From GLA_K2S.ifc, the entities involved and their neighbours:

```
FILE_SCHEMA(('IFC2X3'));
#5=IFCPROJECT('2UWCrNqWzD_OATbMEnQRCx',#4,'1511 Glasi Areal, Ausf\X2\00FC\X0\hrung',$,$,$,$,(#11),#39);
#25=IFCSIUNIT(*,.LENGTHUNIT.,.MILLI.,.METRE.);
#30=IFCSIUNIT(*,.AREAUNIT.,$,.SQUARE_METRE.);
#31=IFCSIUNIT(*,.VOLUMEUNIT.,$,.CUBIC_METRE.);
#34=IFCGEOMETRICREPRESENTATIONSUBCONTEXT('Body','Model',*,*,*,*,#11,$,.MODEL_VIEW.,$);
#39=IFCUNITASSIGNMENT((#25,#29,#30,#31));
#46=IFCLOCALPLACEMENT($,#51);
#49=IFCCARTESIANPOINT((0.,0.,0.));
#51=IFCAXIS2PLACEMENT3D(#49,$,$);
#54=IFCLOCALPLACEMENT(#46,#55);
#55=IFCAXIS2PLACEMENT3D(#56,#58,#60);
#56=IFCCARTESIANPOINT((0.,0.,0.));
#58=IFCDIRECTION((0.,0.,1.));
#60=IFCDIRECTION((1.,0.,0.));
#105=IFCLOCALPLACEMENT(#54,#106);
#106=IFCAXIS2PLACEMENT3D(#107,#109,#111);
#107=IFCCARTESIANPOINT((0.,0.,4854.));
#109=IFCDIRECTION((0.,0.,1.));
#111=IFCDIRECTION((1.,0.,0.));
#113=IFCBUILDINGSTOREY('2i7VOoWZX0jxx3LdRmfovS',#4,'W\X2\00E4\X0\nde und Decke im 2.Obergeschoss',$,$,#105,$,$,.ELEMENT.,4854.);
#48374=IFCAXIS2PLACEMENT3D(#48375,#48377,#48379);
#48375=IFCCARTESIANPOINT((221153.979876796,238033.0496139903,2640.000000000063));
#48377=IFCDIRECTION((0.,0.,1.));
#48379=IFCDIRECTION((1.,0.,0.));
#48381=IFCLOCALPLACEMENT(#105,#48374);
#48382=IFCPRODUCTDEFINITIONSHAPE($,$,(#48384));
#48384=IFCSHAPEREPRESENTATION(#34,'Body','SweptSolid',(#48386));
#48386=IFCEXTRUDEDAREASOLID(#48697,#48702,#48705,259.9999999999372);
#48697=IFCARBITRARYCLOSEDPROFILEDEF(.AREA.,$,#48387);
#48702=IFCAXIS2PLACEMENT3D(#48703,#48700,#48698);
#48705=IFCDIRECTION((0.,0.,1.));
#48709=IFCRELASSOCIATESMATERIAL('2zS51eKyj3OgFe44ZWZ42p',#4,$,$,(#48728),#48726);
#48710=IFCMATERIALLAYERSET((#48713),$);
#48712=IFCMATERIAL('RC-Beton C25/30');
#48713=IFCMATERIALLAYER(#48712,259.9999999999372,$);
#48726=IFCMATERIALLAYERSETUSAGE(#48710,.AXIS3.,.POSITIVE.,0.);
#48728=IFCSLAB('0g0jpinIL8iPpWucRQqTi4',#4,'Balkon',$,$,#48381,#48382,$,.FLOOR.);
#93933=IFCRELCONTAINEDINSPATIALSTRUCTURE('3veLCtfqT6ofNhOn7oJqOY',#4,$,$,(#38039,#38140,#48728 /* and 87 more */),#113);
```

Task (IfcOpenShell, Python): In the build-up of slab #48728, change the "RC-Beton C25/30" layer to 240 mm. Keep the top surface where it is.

```python
import ifcopenshell
import ifcopenshell.util.element
import ifcopenshell.util.representation

model = ifcopenshell.open("GLA_K2S.ifc")

layer_set = model.by_id(48710)
layer = next(l for l in layer_set.MaterialLayers if l.Material and l.Material.Name == "RC-Beton C25/30")
change = 240.0 - layer.LayerThickness
layer.LayerThickness += change

# Geometry does not follow the layer set by itself.
slabs = [e for e in ifcopenshell.util.element.get_elements_by_material(model, layer_set) if e.is_a("IfcSlab")]
for slab in sorted(slabs, key=lambda e: e.id()):
    body = ifcopenshell.util.representation.get_representation(slab, "Model", "Body")
    solid = body.Items[0]
    old_depth = solid.Depth
    solid.Depth += change
    # Extruded upwards: lower the start of the extrusion so the top stays.
    x, y, z = solid.Position.Location.Coordinates
    solid.Position.Location = model.createIfcCartesianPoint((x, y, z - change))
    print(slab.id(), f"{old_depth:g} -> {solid.Depth:g}")

# The layers are counted up from the underside, which has moved.
for usage in {ifcopenshell.util.element.get_material(slab) for slab in slabs}:
    usage.OffsetFromReferenceLine -= change

model.write("GLA_K2S_edited.ifc")
```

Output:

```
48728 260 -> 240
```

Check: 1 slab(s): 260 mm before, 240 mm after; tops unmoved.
